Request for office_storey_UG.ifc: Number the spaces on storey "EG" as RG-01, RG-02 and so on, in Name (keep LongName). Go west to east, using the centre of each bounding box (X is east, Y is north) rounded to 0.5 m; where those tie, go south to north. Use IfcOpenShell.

First a look at what the model holds.

```python
import ifcopenshell
import ifcopenshell.util.element
import ifcopenshell.util.placement

model = ifcopenshell.open("office_storey_UG.ifc")
print(model.schema)
storey = next(s for s in model.by_type("IfcBuildingStorey") if s.Name == "EG")
spaces = [e for e in ifcopenshell.util.element.get_decomposition(storey) if e.is_a("IfcSpace")]
for e in sorted(spaces, key=lambda e: e.id()):
    origin = ifcopenshell.util.placement.get_local_placement(e.ObjectPlacement)[:3, 3]
    print(e.id(), e.Name, e.LongName, origin.round(2) + 0.0, sep=" | ")
```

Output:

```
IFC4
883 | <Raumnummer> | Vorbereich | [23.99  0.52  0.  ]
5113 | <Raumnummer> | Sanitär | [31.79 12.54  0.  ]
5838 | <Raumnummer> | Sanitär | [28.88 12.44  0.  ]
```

```python
import ifcopenshell
import ifcopenshell.geom
import ifcopenshell.util.element
import ifcopenshell.util.shape

model = ifcopenshell.open("office_storey_UG.ifc")
settings = ifcopenshell.geom.settings()
settings.set("use-world-coords", True)


def centre(element):
    shape = ifcopenshell.geom.create_shape(settings, element)
    return ifcopenshell.util.shape.get_bbox_centroid(shape.geometry)


storey = next(s for s in model.by_type("IfcBuildingStorey") if s.Name == "EG")
spaces = [e for e in ifcopenshell.util.element.get_decomposition(storey) if e.is_a("IfcSpace")]

# Insertion points can sit at a corner or the storey origin, so sort by the geometry (in metres).
centres = {e: centre(e) for e in spaces}
spaces.sort(key=lambda e: (round(centres[e][0] / 0.5), centres[e][1]))

for i, e in enumerate(spaces, start=1):
    number = f"RG-{i:02d}"
    e.Name = number
    print(e.id(), number)

model.write("office_storey_UG_edited.ifc")
```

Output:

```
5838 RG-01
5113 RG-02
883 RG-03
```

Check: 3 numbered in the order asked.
